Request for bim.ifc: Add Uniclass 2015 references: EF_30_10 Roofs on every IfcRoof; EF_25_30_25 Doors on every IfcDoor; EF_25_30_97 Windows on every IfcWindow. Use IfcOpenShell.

First a look at what the model holds.

```python
import ifcopenshell

model = ifcopenshell.open("bim.ifc")
print(model.schema)
print("classifications:", [c.Name for c in model.by_type("IfcClassification")])
for ifc_class in ("IfcDoor", "IfcRoof", "IfcStair", "IfcWall", "IfcWindow"):
    print(ifc_class, len(model.by_type(ifc_class)))
```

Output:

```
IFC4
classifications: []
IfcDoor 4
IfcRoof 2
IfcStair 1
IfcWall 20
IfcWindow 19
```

```python
import ifcopenshell
import ifcopenshell.api.classification

model = ifcopenshell.open("bim.ifc")

system = ifcopenshell.api.classification.add_classification(model, classification="Uniclass 2015")

codes = {
    "IfcRoof": ("EF_30_10", "Roofs"),
    "IfcDoor": ("EF_25_30_25", "Doors"),
    "IfcWindow": ("EF_25_30_97", "Windows"),
}
for ifc_class, (code, name) in codes.items():
    products = model.by_type(ifc_class)
    ifcopenshell.api.classification.add_reference(
        model, products=products, classification=system, identification=code, name=name
    )
    print(code, len(products))

model.write("bim_v2.ifc")
```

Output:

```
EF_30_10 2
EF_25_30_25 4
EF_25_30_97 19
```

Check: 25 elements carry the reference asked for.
